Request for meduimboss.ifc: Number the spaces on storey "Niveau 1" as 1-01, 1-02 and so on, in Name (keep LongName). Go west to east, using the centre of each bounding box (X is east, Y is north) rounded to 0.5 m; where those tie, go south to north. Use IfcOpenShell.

First a look at what the model holds.

```python
import ifcopenshell
import ifcopenshell.util.element
import ifcopenshell.util.placement

model = ifcopenshell.open("meduimboss.ifc")
print(model.schema)
storey = next(s for s in model.by_type("IfcBuildingStorey") if s.Name == "Niveau 1")
spaces = [e for e in ifcopenshell.util.element.get_decomposition(storey) if e.is_a("IfcSpace")]
for e in sorted(spaces, key=lambda e: e.id()):
    origin = ifcopenshell.util.placement.get_local_placement(e.ObjectPlacement)[:3, 3]
    print(e.id(), e.Name, e.LongName, origin.round(2) + 0.0, sep=" | ")
```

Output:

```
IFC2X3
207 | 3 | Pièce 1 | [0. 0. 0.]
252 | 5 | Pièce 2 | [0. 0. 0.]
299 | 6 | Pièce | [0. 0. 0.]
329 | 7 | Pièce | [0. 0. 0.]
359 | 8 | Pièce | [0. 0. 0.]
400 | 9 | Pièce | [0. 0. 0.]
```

```python
import ifcopenshell
import ifcopenshell.geom
import ifcopenshell.util.element
import ifcopenshell.util.shape

model = ifcopenshell.open("meduimboss.ifc")
settings = ifcopenshell.geom.settings()
settings.set("use-world-coords", True)


def centre(element):
    shape = ifcopenshell.geom.create_shape(settings, element)
    return ifcopenshell.util.shape.get_bbox_centroid(shape.geometry)


storey = next(s for s in model.by_type("IfcBuildingStorey") if s.Name == "Niveau 1")
spaces = [e for e in ifcopenshell.util.element.get_decomposition(storey) if e.is_a("IfcSpace")]

# Insertion points can sit at a corner or the storey origin, so sort by the geometry (in metres).
centres = {e: centre(e) for e in spaces}
spaces.sort(key=lambda e: (round(centres[e][0] / 0.5), centres[e][1]))

for i, e in enumerate(spaces, start=1):
    number = f"1-{i:02d}"
    e.Name = number
    print(e.id(), number)

model.write("meduimboss_v2.ifc")
```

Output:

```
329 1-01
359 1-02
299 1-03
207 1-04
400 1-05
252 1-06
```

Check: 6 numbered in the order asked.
